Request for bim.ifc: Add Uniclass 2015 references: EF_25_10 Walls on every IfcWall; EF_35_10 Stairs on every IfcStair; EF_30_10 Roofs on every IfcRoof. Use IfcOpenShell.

First a look at what the model holds.

```python
import ifcopenshell

model = ifcopenshell.open("bim.ifc")
print(model.schema)
print("classifications:", [c.Name for c in model.by_type("IfcClassification")])
for ifc_class in ("IfcDoor", "IfcRoof", "IfcStair", "IfcWall", "IfcWindow"):
    print(ifc_class, len(model.by_type(ifc_class)))
```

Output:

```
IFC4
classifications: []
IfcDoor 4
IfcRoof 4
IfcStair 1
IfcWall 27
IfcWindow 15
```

```python
import ifcopenshell
import ifcopenshell.api.classification

model = ifcopenshell.open("bim.ifc")

system = ifcopenshell.api.classification.add_classification(model, classification="Uniclass 2015")

codes = {
    "IfcWall": ("EF_25_10", "Walls"),
    "IfcStair": ("EF_35_10", "Stairs"),
    "IfcRoof": ("EF_30_10", "Roofs"),
}
for ifc_class, (code, name) in codes.items():
    products = model.by_type(ifc_class)
    ifcopenshell.api.classification.add_reference(
        model, products=products, classification=system, identification=code, name=name
    )
    print(code, len(products))

model.write("bim_v2.ifc")
```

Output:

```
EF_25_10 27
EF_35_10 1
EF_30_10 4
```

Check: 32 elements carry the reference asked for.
